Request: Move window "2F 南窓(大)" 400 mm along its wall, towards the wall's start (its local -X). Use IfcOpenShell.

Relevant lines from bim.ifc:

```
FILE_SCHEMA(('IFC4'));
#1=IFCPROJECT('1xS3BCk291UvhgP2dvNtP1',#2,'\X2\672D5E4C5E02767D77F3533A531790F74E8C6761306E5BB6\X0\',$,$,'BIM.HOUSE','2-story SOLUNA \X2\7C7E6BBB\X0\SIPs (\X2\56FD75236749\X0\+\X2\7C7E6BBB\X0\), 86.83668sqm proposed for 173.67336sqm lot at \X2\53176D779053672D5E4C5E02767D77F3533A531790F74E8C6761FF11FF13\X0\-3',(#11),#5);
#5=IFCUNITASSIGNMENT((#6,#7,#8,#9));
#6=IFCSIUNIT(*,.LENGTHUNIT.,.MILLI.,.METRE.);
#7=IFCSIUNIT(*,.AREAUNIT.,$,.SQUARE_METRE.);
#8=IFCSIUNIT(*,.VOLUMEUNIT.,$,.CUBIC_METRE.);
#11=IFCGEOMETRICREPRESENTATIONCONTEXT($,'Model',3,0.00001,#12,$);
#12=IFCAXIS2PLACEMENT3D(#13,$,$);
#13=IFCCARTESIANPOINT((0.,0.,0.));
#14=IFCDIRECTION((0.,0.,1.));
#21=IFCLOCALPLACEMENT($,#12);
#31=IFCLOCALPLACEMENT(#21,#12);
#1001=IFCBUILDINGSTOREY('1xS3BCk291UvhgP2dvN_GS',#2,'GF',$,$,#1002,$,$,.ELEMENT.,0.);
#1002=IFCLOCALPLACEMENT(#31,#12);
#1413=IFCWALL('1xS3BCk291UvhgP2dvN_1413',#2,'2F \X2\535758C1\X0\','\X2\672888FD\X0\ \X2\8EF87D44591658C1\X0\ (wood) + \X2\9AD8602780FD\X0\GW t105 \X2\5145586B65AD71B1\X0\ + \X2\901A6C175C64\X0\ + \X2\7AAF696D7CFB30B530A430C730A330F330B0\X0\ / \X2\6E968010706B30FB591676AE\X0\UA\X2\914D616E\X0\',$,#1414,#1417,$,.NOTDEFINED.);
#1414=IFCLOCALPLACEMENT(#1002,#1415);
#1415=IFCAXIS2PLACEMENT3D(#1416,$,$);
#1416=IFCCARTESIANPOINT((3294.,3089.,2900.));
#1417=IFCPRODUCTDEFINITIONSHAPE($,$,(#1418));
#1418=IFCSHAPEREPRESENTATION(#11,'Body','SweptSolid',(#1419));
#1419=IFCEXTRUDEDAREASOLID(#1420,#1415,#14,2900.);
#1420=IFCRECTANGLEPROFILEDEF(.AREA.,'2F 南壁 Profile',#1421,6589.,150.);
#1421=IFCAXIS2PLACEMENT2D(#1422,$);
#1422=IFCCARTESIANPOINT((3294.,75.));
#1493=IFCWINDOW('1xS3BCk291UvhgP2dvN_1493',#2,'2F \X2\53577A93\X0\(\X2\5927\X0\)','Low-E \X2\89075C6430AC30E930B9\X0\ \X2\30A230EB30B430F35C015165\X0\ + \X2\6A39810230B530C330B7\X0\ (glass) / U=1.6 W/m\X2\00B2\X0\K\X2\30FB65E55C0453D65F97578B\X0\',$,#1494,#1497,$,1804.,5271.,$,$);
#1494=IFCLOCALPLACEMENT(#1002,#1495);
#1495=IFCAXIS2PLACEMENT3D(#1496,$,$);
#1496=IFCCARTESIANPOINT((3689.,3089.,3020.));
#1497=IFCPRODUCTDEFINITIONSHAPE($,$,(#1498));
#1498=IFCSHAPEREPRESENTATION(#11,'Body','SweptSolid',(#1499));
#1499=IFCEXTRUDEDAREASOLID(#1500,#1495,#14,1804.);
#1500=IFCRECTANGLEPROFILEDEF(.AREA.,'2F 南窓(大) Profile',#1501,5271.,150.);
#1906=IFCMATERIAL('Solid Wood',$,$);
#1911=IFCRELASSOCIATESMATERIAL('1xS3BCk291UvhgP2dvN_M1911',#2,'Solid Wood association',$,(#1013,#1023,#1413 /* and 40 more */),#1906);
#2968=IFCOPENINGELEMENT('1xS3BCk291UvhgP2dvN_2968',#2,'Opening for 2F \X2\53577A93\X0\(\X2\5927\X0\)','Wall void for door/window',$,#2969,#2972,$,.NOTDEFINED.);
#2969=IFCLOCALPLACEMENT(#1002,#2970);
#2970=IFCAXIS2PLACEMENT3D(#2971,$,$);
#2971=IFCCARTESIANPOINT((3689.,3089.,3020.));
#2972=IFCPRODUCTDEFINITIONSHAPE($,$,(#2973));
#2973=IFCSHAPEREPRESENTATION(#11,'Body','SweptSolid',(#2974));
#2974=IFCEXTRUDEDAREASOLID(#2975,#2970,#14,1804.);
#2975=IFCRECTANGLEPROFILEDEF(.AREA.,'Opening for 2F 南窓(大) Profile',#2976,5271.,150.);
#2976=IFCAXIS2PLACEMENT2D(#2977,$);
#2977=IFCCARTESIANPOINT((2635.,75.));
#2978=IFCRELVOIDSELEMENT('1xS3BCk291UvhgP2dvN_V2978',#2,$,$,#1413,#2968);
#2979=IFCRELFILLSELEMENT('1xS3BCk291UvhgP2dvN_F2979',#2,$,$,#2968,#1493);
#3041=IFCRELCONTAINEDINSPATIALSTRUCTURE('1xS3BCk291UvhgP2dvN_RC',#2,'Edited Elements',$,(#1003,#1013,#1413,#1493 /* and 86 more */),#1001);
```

```python
import ifcopenshell
import ifcopenshell.api.geometry
import ifcopenshell.util.placement
import ifcopenshell.util.unit

model = ifcopenshell.open("bim.ifc")
unit_scale = ifcopenshell.util.unit.calculate_unit_scale(model)

window = model.by_guid("1xS3BCk291UvhgP2dvN_1493")
opening = window.FillsVoids[0].RelatingOpeningElement
wall = opening.VoidsElements[0].RelatingBuildingElement

wall_matrix = ifcopenshell.util.placement.get_local_placement(wall.ObjectPlacement)
shift = wall_matrix[:3, 0] * -0.4 / unit_scale
before = ifcopenshell.util.placement.get_local_placement(window.ObjectPlacement)[:3, 3].copy()

# The window is not placed relative to its opening, so move both.
for product in (opening, window):
    matrix = ifcopenshell.util.placement.get_local_placement(product.ObjectPlacement)
    matrix[:3, 3] += shift
    ifcopenshell.api.geometry.edit_object_placement(model, product=product, matrix=matrix, is_si=False)

after = ifcopenshell.util.placement.get_local_placement(window.ObjectPlacement)[:3, 3]
print("window moved by", (after - before).round(3) + 0.0)

model.write("bim_updated.ifc")
```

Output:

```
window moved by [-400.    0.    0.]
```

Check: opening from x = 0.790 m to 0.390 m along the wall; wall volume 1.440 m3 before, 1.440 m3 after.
